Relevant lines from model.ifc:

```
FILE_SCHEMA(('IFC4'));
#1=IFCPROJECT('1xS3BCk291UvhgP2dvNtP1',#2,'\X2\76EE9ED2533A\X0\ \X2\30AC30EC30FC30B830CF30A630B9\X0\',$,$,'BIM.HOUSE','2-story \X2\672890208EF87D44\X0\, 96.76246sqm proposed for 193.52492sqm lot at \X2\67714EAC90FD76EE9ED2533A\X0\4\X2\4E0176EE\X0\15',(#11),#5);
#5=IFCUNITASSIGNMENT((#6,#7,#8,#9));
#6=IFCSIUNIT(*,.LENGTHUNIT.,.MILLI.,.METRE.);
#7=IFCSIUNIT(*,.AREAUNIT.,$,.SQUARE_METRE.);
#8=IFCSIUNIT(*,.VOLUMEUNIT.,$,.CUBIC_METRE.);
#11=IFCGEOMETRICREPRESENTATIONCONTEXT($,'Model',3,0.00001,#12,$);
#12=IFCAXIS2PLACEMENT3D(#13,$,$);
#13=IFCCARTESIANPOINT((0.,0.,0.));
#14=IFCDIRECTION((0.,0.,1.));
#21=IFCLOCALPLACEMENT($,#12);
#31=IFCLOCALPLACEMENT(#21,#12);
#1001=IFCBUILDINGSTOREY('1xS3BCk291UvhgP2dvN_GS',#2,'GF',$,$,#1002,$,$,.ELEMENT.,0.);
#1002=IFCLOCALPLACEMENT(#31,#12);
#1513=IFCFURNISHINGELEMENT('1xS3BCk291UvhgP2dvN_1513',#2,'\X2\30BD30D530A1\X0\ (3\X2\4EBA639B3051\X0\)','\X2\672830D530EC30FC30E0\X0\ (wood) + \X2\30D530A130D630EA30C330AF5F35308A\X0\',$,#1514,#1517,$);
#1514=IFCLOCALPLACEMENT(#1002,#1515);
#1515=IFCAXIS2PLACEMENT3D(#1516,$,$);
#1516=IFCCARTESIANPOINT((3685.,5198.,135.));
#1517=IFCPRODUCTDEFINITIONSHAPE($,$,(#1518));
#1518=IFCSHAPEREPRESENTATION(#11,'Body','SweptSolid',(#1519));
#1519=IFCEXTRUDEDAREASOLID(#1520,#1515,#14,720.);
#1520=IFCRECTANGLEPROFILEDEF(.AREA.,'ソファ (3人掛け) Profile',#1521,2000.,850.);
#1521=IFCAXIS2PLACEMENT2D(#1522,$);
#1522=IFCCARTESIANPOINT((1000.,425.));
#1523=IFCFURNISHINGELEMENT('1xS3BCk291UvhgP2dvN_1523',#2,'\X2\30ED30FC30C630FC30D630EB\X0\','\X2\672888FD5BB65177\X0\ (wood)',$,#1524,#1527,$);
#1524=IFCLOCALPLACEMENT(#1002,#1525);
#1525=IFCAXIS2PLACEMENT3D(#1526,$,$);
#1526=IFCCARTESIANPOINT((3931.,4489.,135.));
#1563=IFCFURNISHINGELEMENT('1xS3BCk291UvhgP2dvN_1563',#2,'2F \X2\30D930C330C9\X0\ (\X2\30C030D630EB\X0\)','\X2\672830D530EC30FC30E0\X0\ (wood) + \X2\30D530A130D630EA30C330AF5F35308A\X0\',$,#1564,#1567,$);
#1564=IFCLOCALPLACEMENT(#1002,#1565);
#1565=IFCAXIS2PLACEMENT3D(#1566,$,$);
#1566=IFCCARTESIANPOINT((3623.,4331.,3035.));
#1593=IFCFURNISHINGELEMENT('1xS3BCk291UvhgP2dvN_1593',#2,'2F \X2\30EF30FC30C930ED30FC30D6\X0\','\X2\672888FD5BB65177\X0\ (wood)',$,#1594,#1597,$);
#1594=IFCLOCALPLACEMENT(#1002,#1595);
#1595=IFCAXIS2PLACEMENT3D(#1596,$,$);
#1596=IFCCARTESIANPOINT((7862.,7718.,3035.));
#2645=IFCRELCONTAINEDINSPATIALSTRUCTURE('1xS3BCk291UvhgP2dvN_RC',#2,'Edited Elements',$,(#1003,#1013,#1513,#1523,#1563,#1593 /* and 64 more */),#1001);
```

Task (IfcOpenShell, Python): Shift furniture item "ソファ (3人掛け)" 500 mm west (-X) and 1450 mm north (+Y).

```python
import ifcopenshell
import ifcopenshell.api.geometry
import ifcopenshell.util.placement
import ifcopenshell.util.unit

model = ifcopenshell.open("model.ifc")
unit_scale = ifcopenshell.util.unit.calculate_unit_scale(model)

item = model.by_guid("1xS3BCk291UvhgP2dvN_1513")
matrix = ifcopenshell.util.placement.get_local_placement(item.ObjectPlacement)
matrix[0, 3] -= 0.5 / unit_scale
matrix[1, 3] += 1.45 / unit_scale
ifcopenshell.api.geometry.edit_object_placement(model, product=item, matrix=matrix, is_si=False)

print(ifcopenshell.util.placement.get_local_placement(item.ObjectPlacement).round(3) + 0.0)

model.write("model_edited.ifc")
```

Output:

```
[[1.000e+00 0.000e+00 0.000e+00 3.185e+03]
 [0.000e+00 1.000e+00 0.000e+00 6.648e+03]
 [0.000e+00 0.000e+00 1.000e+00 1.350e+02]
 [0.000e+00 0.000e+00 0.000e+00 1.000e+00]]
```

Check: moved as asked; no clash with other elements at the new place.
